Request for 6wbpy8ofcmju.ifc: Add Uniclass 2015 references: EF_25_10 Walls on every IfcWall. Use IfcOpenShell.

First a look at what the model holds.

```python
import ifcopenshell

model = ifcopenshell.open("6wbpy8ofcmju.ifc")
print(model.schema)
print("classifications:", [c.Name for c in model.by_type("IfcClassification")])
for ifc_class in ("IfcDoor", "IfcRoof", "IfcStair", "IfcWall", "IfcWindow"):
    print(ifc_class, len(model.by_type(ifc_class)))
```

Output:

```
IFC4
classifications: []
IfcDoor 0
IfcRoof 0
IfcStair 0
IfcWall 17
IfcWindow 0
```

```python
import ifcopenshell
import ifcopenshell.api.classification

model = ifcopenshell.open("6wbpy8ofcmju.ifc")

system = ifcopenshell.api.classification.add_classification(model, classification="Uniclass 2015")

codes = {
    "IfcWall": ("EF_25_10", "Walls"),
}
for ifc_class, (code, name) in codes.items():
    products = model.by_type(ifc_class)
    ifcopenshell.api.classification.add_reference(
        model, products=products, classification=system, identification=code, name=name
    )
    print(code, len(products))

model.write("6wbpy8ofcmju_rev.ifc")
```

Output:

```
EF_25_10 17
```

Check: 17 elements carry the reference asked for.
